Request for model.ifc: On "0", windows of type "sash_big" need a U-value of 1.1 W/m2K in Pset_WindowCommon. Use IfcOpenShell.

First a look at what the model holds.

```python
import ifcopenshell
import ifcopenshell.util.element

model = ifcopenshell.open("model.ifc")
print(model.schema)
storey = next(s for s in model.by_type("IfcBuildingStorey") if s.Name == "0")
windows = [e for e in ifcopenshell.util.element.get_decomposition(storey) if e.is_a("IfcWindow")]
seen = {}
for e in windows:
    element_type = ifcopenshell.util.element.get_type(e)
    key = (element_type.Name if element_type != e and element_type else None, ifcopenshell.util.element.get_pset(e, "Pset_WindowCommon", "ThermalTransmittance"))
    seen[key] = seen.get(key, 0) + 1
for (name, value), count in sorted(seen.items(), key=str):
    print(count, "x", name, "|", value)
```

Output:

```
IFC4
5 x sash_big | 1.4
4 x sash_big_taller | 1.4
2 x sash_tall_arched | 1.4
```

```python
import ifcopenshell
import ifcopenshell.api.pset
import ifcopenshell.util.element

model = ifcopenshell.open("model.ifc")

storey = next(s for s in model.by_type("IfcBuildingStorey") if s.Name == "0")
windows = [e for e in ifcopenshell.util.element.get_decomposition(storey) if e.is_a("IfcWindow")]

count = 0
for e in windows:
    element_type = ifcopenshell.util.element.get_type(e)
    if element_type in (None, e) or element_type.Name != "sash_big":
        continue
    # add_pset returns the element's existing set when there is one.
    pset = ifcopenshell.api.pset.add_pset(model, product=e, name="Pset_WindowCommon")
    ifcopenshell.api.pset.edit_pset(model, pset=pset, properties={"ThermalTransmittance": 1.1})
    count += 1

print(count, "windows updated")

model.write("model_v2.ifc")
```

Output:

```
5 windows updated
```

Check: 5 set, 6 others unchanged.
